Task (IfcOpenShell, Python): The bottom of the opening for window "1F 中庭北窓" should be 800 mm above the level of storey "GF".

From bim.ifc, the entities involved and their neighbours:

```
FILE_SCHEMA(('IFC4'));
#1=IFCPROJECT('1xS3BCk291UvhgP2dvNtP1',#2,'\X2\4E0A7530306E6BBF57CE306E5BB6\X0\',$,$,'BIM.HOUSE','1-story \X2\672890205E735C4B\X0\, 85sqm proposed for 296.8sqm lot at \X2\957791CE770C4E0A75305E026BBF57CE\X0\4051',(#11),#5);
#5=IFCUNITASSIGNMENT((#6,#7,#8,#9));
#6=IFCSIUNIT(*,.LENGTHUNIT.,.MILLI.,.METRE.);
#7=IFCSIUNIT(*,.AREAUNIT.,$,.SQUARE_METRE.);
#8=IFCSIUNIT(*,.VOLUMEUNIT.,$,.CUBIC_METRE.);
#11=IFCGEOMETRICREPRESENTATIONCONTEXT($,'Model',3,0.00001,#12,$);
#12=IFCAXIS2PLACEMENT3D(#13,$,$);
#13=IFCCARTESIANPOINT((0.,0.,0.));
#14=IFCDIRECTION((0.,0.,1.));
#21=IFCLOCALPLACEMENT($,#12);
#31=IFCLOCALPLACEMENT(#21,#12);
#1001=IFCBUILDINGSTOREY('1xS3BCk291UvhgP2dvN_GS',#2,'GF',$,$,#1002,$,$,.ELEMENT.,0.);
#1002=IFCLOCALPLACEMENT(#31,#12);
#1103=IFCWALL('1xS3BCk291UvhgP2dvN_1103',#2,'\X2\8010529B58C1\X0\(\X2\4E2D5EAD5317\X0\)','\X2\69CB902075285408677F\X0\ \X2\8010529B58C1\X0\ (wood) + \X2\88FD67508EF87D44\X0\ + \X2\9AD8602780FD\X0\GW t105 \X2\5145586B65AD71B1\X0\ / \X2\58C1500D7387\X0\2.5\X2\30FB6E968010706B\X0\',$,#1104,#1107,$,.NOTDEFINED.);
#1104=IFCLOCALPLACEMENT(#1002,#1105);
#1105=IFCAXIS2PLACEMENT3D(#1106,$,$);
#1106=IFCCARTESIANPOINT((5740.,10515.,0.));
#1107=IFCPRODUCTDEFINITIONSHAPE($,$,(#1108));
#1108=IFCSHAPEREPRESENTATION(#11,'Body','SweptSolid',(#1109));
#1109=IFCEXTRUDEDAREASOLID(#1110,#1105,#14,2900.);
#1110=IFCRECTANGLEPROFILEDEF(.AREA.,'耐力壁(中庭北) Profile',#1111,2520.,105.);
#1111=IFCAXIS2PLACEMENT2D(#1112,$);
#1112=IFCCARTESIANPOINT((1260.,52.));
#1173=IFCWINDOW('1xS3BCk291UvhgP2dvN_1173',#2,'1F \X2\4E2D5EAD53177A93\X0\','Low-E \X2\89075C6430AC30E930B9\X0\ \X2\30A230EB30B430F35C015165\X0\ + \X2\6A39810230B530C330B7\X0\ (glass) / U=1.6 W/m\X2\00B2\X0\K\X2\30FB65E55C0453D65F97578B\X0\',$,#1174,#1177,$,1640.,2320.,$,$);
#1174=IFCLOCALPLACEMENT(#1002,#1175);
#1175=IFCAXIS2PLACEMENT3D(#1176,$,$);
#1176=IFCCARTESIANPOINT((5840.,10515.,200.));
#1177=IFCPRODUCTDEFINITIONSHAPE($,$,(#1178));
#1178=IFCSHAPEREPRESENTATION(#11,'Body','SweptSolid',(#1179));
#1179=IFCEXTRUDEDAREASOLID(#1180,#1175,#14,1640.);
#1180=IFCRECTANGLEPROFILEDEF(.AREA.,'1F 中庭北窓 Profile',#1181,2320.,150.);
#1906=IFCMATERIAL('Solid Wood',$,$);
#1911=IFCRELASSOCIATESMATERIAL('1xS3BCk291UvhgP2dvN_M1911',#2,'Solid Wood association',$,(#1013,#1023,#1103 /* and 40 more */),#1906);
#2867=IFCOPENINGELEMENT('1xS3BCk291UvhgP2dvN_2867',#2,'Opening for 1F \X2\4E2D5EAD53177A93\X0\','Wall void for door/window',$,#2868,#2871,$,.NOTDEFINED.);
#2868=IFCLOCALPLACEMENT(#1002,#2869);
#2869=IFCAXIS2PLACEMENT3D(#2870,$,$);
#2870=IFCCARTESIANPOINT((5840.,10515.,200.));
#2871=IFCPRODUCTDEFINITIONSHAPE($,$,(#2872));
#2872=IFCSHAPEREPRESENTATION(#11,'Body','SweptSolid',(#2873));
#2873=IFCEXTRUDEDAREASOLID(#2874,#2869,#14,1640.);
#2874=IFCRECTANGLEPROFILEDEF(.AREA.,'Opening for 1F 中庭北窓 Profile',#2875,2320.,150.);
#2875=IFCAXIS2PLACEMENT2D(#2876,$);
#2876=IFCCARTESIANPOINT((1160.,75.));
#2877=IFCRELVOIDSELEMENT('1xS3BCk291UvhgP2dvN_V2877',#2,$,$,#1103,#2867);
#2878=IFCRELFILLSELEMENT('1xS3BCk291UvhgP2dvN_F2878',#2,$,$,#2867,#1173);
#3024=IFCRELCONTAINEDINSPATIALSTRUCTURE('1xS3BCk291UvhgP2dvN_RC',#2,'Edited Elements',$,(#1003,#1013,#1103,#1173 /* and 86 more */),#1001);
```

```python
import numpy as np
import ifcopenshell
import ifcopenshell.api.geometry
import ifcopenshell.geom
import ifcopenshell.util.element
import ifcopenshell.util.placement
import ifcopenshell.util.shape
import ifcopenshell.util.unit

model = ifcopenshell.open("bim.ifc")
unit_scale = ifcopenshell.util.unit.calculate_unit_scale(model)

window = model.by_guid("1xS3BCk291UvhgP2dvN_1173")
opening = window.FillsVoids[0].RelatingOpeningElement
storey = ifcopenshell.util.element.get_container(window, ifc_class="IfcBuildingStorey")
level = ifcopenshell.util.placement.get_local_placement(storey.ObjectPlacement)[2, 3]

# The opening's origin need not be at the sill, so measure its lowest point.
shape = ifcopenshell.geom.create_shape(ifcopenshell.geom.settings(), opening)
bottom = ifcopenshell.util.shape.get_shape_bottom_elevation(shape, shape.geometry) / unit_scale
dz = level + 0.8 / unit_scale - bottom

shift = np.array([0.0, 0.0, dz])
# The window is not placed relative to its opening, so move both.
for product in (opening, window):
    matrix = ifcopenshell.util.placement.get_local_placement(product.ObjectPlacement)
    matrix[:3, 3] += shift
    ifcopenshell.api.geometry.edit_object_placement(model, product=product, matrix=matrix, is_si=False)

print(f"moved by {dz * unit_scale:+.3f} m")

model.write("bim_edited.ifc")
```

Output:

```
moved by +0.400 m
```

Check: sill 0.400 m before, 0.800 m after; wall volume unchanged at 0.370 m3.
